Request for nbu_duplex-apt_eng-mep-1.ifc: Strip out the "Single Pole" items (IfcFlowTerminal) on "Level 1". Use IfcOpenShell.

First a look at what the model holds.

```python
import ifcopenshell
import ifcopenshell.util.element

model = ifcopenshell.open("nbu_duplex-apt_eng-mep-1.ifc")
print(model.schema)
storey = next(s for s in model.by_type("IfcBuildingStorey") if s.Name == "Level 1")
terminals = [e for e in ifcopenshell.util.element.get_decomposition(storey) if e.is_a("IfcFlowTerminal")]
seen = {}
for e in terminals:
    element_type = ifcopenshell.util.element.get_type(e)
    name = element_type.Name if element_type not in (None, e) else None
    seen[name] = seen.get(name, 0) + 1
for name, count in sorted(seen.items(), key=str):
    print(count, "x", name)
```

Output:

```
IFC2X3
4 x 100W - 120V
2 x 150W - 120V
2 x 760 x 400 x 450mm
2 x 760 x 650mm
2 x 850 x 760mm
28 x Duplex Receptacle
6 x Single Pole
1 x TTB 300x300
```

```python
import ifcopenshell
import ifcopenshell.api.root
import ifcopenshell.util.element

model = ifcopenshell.open("nbu_duplex-apt_eng-mep-1.ifc")

storey = next(s for s in model.by_type("IfcBuildingStorey") if s.Name == "Level 1")
terminals = [e for e in ifcopenshell.util.element.get_decomposition(storey) if e.is_a("IfcFlowTerminal")]
targets = [e for e in terminals if (t := ifcopenshell.util.element.get_type(e)) not in (None, e) and t.Name == "Single Pole"]

for e in targets:
    ifcopenshell.api.root.remove_product(model, product=e)
print(len(targets), "removed")

model.write("nbu_duplex-apt_eng-mep-1_v2.ifc")
```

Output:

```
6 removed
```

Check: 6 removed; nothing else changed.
